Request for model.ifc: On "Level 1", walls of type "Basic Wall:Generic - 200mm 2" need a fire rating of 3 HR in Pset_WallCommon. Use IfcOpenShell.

First a look at what the model holds.

```python
import ifcopenshell
import ifcopenshell.util.element

model = ifcopenshell.open("model.ifc")
print(model.schema)
storey = next(s for s in model.by_type("IfcBuildingStorey") if s.Name == "Level 1")
walls = [e for e in ifcopenshell.util.element.get_decomposition(storey) if e.is_a("IfcWall")]
seen = {}
for e in walls:
    element_type = ifcopenshell.util.element.get_type(e)
    key = (element_type.Name if element_type != e and element_type else None, ifcopenshell.util.element.get_pset(e, "Pset_WallCommon", "FireRating"))
    seen[key] = seen.get(key, 0) + 1
for (name, value), count in sorted(seen.items(), key=str):
    print(count, "x", name, "|", value)
```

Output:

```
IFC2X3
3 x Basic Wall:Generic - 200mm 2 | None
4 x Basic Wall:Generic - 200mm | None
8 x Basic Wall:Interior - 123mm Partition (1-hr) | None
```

```python
import ifcopenshell
import ifcopenshell.api.pset
import ifcopenshell.util.element

model = ifcopenshell.open("model.ifc")

storey = next(s for s in model.by_type("IfcBuildingStorey") if s.Name == "Level 1")
walls = [e for e in ifcopenshell.util.element.get_decomposition(storey) if e.is_a("IfcWall")]

count = 0
for e in walls:
    element_type = ifcopenshell.util.element.get_type(e)
    if element_type in (None, e) or element_type.Name != "Basic Wall:Generic - 200mm 2":
        continue
    found = ifcopenshell.util.element.get_pset(e, "Pset_WallCommon", should_inherit=False)
    if found:
        pset = model.by_id(found["id"])
        if len(ifcopenshell.util.element.get_elements_by_pset(pset)) > 1:
            pset = ifcopenshell.api.pset.unshare_pset(model, products=[e], pset=pset)[0]
    else:
        pset = ifcopenshell.api.pset.add_pset(model, product=e, name="Pset_WallCommon")
    ifcopenshell.api.pset.edit_pset(model, pset=pset, properties={"FireRating": "3 HR"})
    count += 1

print(count, "walls updated")

model.write("model_edited.ifc")
```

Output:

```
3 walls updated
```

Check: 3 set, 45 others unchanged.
